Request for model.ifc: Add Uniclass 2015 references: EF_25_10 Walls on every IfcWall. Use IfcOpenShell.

First a look at what the model holds.

```python
import ifcopenshell

model = ifcopenshell.open("model.ifc")
print(model.schema)
print("classifications:", [c.Name for c in model.by_type("IfcClassification")])
for ifc_class in ("IfcDoor", "IfcRoof", "IfcStair", "IfcWall", "IfcWindow"):
    print(ifc_class, len(model.by_type(ifc_class)))
```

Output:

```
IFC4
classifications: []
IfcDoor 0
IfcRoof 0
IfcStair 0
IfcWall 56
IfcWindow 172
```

```python
import ifcopenshell
import ifcopenshell.api.classification

model = ifcopenshell.open("model.ifc")

system = ifcopenshell.api.classification.add_classification(model, classification="Uniclass 2015")

codes = {
    "IfcWall": ("EF_25_10", "Walls"),
}
for ifc_class, (code, name) in codes.items():
    products = model.by_type(ifc_class)
    ifcopenshell.api.classification.add_reference(
        model, products=products, classification=system, identification=code, name=name
    )
    print(code, len(products))

model.write("model_edited.ifc")
```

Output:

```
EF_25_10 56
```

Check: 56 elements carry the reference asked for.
